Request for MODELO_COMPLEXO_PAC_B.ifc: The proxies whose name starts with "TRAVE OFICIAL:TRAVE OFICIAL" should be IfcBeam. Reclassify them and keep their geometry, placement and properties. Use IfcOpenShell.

First a look at what the model holds.

```python
import re

import ifcopenshell

model = ifcopenshell.open("MODELO_COMPLEXO_PAC_B.ifc")
print(model.schema)
seen = {}
for e in model.by_type("IfcBuildingElementProxy"):
    name = re.sub(r":\d+(:\d+)?$", "", e.Name or "")  # drop the element id that some exporters append
    seen[name] = seen.get(name, 0) + 1
for name, count in sorted(seen.items()):
    print(count, "x", name)
```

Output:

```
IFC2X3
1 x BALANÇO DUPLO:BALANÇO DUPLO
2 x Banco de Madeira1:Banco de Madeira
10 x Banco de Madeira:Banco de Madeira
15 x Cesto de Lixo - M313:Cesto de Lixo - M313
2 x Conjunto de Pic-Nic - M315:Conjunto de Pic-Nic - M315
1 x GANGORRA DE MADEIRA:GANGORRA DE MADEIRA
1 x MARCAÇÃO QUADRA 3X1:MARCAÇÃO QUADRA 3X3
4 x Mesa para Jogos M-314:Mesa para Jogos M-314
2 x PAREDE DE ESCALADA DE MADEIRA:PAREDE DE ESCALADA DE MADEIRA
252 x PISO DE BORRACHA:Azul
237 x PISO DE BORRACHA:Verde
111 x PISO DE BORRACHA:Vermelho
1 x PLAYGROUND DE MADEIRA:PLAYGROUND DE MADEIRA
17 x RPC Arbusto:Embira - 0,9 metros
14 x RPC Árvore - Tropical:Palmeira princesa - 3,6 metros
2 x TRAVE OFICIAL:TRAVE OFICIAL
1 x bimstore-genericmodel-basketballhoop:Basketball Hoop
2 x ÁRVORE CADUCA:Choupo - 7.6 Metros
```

```python
import ifcopenshell
import ifcopenshell.api.root

model = ifcopenshell.open("MODELO_COMPLEXO_PAC_B.ifc")

proxies = [e.id() for e in model.by_type("IfcBuildingElementProxy") if (e.Name or "").startswith("TRAVE OFICIAL:TRAVE OFICIAL")]
for step_id in proxies:
    proxy = model.by_id(step_id)
    # Reclassifying a typed element also reclassifies its type and the type's other occurrences.
    if proxy.is_a("IfcBuildingElementProxy"):
        ifcopenshell.api.root.reassign_class(model, product=proxy, ifc_class="IfcBeam")

print(sum(model.by_id(i).is_a("IfcBeam") for i in proxies), "reclassified")

model.write("MODELO_COMPLEXO_PAC_B_updated.ifc")
```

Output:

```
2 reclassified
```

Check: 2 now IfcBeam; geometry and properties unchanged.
